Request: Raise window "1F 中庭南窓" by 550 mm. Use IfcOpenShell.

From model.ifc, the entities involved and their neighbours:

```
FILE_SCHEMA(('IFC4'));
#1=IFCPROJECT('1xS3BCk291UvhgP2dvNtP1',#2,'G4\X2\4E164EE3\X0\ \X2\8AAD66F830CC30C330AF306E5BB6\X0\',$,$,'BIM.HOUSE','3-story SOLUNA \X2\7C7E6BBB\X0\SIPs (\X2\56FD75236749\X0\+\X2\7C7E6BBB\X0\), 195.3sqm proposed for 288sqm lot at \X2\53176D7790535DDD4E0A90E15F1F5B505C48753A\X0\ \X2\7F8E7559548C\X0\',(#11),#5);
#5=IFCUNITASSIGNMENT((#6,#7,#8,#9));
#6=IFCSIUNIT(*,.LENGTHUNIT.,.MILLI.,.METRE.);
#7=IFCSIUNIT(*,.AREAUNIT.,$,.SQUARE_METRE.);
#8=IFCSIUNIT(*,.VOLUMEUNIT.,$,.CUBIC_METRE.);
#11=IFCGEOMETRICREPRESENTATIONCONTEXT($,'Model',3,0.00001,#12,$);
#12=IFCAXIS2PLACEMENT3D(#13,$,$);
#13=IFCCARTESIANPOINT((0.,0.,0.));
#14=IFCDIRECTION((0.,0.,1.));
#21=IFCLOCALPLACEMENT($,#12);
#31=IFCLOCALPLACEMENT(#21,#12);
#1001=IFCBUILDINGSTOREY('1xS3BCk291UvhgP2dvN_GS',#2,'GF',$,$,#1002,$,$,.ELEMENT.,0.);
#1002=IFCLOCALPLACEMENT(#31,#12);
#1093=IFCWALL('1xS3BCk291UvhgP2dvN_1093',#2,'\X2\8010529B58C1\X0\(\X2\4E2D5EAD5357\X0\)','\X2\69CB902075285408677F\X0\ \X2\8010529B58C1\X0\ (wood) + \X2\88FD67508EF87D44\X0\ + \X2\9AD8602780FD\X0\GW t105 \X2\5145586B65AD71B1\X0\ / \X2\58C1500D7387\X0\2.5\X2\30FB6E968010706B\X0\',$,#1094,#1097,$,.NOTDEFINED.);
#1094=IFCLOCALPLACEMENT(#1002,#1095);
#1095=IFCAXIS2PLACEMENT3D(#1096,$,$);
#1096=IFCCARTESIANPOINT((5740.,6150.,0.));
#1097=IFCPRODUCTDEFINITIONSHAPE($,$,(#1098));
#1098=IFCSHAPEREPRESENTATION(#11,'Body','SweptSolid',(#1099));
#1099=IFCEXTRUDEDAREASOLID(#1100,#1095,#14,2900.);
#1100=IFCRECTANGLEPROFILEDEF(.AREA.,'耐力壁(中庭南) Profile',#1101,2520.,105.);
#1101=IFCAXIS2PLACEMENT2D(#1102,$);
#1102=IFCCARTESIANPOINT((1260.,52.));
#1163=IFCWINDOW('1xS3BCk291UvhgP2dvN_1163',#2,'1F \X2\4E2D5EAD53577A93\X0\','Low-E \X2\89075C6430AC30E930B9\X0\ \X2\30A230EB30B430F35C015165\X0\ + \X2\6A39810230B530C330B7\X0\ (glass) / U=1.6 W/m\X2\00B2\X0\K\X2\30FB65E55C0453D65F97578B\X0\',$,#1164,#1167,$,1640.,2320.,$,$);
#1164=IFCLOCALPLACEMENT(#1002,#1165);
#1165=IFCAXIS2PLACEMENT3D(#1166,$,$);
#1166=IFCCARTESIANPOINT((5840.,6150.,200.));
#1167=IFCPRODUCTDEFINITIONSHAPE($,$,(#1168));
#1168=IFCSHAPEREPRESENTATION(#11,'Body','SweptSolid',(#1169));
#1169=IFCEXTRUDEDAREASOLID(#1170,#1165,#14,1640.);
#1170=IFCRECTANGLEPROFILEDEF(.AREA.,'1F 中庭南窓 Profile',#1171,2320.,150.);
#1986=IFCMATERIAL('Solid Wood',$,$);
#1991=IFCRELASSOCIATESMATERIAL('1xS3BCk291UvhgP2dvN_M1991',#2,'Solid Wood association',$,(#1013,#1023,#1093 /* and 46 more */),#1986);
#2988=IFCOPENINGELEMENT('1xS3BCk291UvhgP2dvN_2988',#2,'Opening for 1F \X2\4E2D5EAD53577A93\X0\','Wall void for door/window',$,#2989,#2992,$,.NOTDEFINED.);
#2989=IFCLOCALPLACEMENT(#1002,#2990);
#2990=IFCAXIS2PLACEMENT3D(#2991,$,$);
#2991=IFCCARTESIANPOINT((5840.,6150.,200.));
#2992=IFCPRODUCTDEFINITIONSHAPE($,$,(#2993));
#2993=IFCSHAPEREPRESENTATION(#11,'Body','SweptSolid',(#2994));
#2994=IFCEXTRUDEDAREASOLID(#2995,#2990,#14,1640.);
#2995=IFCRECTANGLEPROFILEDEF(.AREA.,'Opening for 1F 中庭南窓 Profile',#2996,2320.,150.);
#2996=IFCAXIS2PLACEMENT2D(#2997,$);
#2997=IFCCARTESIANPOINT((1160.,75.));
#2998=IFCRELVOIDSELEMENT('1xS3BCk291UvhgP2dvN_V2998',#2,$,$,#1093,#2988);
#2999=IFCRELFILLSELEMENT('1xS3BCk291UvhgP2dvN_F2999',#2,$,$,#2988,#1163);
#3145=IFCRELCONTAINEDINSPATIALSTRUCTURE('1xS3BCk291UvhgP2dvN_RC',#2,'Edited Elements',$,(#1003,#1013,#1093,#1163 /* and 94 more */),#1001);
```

```python
import numpy as np
import ifcopenshell
import ifcopenshell.api.geometry
import ifcopenshell.util.placement
import ifcopenshell.util.unit

model = ifcopenshell.open("model.ifc")
unit_scale = ifcopenshell.util.unit.calculate_unit_scale(model)

window = model.by_id(1163)
opening = window.FillsVoids[0].RelatingOpeningElement
dz = 0.55 / unit_scale

shift = np.array([0.0, 0.0, dz])
# The window is not placed relative to its opening, so move both.
for product in (opening, window):
    matrix = ifcopenshell.util.placement.get_local_placement(product.ObjectPlacement)
    matrix[:3, 3] += shift
    ifcopenshell.api.geometry.edit_object_placement(model, product=product, matrix=matrix, is_si=False)

print(f"moved by {dz * unit_scale:+.3f} m")

model.write("model_updated.ifc")
```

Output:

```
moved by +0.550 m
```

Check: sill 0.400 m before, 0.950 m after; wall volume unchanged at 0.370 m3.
